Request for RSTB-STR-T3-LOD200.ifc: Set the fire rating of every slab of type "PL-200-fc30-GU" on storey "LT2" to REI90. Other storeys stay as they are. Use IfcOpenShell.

First a look at what the model holds.

```python
import ifcopenshell
import ifcopenshell.util.element

model = ifcopenshell.open("RSTB-STR-T3-LOD200.ifc")
print(model.schema)
storey = next(s for s in model.by_type("IfcBuildingStorey") if s.Name == "LT2")
slabs = [e for e in ifcopenshell.util.element.get_decomposition(storey) if e.is_a("IfcSlab")]
seen = {}
for e in slabs:
    element_type = ifcopenshell.util.element.get_type(e)
    key = (element_type.Name if element_type != e and element_type else None, ifcopenshell.util.element.get_pset(e, "Pset_SlabCommon", "FireRating"))
    seen[key] = seen.get(key, 0) + 1
for (name, value), count in sorted(seen.items(), key=str):
    print(count, "x", name, "|", value)
```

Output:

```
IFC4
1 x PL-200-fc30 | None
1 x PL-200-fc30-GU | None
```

```python
import ifcopenshell
import ifcopenshell.api.pset
import ifcopenshell.util.element

model = ifcopenshell.open("RSTB-STR-T3-LOD200.ifc")

storey = next(s for s in model.by_type("IfcBuildingStorey") if s.Name == "LT2")
slabs = [e for e in ifcopenshell.util.element.get_decomposition(storey) if e.is_a("IfcSlab")]

count = 0
for e in slabs:
    element_type = ifcopenshell.util.element.get_type(e)
    if element_type in (None, e) or element_type.Name != "PL-200-fc30-GU":
        continue
    # add_pset returns the element's existing set when there is one.
    pset = ifcopenshell.api.pset.add_pset(model, product=e, name="Pset_SlabCommon")
    ifcopenshell.api.pset.edit_pset(model, pset=pset, properties={"FireRating": "REI90"})
    count += 1

print(count, "slabs updated")

model.write("RSTB-STR-T3-LOD200_v2.ifc")
```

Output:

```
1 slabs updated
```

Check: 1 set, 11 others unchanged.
